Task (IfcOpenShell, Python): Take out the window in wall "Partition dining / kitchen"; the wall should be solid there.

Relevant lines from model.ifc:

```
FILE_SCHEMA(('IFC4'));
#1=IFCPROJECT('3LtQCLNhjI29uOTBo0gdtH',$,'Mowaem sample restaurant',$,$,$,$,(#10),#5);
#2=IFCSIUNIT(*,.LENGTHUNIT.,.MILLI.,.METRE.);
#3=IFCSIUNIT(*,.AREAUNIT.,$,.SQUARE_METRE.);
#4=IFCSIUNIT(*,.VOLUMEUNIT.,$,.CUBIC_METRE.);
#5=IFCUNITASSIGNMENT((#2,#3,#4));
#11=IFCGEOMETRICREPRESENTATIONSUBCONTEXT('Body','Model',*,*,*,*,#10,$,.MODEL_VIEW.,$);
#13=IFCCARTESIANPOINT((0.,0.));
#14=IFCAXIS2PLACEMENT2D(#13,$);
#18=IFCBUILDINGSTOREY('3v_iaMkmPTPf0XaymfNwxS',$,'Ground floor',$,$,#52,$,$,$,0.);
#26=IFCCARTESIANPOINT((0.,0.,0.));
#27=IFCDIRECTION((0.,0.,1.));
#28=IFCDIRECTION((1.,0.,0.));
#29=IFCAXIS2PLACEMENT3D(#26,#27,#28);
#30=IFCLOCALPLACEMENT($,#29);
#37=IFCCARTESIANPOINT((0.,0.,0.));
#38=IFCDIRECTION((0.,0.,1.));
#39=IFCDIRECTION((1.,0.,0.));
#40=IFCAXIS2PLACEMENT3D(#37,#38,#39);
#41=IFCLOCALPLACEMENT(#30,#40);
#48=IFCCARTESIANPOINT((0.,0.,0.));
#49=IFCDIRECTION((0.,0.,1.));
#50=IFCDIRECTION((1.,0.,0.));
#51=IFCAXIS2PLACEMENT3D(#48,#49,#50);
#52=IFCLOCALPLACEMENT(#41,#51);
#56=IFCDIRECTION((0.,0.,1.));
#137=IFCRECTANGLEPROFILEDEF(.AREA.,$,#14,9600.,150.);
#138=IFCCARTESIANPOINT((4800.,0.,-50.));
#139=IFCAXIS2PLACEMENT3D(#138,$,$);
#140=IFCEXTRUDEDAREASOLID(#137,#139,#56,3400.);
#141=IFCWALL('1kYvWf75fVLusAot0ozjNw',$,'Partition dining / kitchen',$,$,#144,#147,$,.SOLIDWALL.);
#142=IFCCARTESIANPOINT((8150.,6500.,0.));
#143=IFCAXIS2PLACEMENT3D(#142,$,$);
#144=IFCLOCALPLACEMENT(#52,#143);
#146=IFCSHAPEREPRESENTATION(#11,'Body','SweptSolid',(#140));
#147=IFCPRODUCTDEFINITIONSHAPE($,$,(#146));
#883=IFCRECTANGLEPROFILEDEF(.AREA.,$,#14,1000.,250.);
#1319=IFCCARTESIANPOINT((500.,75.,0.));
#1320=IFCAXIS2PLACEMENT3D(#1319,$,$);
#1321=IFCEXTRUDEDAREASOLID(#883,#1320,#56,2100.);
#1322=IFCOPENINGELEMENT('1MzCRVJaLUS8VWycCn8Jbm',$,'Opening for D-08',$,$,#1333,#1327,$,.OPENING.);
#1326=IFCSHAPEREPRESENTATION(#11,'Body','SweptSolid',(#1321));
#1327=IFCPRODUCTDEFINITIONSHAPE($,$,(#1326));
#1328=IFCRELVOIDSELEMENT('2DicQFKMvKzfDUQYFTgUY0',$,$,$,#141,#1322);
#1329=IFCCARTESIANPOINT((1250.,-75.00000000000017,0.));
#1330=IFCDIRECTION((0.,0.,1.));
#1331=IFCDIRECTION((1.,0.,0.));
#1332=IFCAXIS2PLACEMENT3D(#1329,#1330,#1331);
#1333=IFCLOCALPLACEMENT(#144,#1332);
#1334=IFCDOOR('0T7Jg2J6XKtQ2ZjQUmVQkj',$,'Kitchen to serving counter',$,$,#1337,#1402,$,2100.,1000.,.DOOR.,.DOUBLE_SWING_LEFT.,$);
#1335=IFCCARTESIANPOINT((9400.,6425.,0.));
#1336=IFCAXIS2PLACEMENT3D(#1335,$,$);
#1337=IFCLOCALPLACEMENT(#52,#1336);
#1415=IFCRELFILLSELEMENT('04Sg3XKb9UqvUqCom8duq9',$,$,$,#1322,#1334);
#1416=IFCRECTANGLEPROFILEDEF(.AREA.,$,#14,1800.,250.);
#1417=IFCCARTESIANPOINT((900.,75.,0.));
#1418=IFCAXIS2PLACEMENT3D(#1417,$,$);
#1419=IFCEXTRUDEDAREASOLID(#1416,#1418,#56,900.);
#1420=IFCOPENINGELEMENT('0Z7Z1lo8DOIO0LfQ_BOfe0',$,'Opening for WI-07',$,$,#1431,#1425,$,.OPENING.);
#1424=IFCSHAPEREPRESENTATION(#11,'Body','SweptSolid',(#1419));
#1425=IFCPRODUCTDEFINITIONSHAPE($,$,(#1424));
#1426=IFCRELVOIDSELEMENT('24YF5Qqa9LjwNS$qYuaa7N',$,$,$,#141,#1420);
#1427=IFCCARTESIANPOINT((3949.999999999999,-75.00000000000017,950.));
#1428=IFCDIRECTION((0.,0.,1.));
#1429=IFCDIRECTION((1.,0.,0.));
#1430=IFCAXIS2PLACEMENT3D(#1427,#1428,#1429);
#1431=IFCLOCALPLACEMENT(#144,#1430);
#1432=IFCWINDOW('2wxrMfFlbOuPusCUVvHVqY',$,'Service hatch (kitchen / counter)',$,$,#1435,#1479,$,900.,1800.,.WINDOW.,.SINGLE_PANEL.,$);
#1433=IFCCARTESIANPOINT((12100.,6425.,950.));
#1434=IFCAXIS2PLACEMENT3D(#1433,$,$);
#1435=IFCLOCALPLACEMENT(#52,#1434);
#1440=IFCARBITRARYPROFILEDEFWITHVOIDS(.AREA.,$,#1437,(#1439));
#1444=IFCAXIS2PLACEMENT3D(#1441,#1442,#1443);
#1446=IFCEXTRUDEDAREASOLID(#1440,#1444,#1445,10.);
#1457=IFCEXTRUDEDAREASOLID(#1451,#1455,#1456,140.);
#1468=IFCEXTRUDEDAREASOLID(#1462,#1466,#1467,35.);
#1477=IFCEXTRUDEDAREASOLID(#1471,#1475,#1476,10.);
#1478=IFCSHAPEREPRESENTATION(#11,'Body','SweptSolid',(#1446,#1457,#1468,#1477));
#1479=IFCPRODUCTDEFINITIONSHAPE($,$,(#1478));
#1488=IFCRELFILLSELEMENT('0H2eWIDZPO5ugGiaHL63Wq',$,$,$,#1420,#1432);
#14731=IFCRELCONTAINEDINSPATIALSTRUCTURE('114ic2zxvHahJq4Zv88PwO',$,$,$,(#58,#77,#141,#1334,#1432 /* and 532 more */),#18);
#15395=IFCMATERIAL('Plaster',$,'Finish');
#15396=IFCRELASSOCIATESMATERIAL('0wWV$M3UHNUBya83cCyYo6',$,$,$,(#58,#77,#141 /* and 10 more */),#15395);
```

```python
import ifcopenshell
import ifcopenshell.api.feature
import ifcopenshell.api.root
import ifcopenshell.geom
import ifcopenshell.util.shape

model = ifcopenshell.open("model.ifc")
settings = ifcopenshell.geom.settings()


def volume(element):
    """Net volume in cubic metres, openings subtracted."""
    shape = ifcopenshell.geom.create_shape(settings, element)
    return ifcopenshell.util.shape.get_volume(shape.geometry)


window = model.by_guid("2wxrMfFlbOuPusCUVvHVqY")
opening = window.FillsVoids[0].RelatingOpeningElement
wall = opening.VoidsElements[0].RelatingBuildingElement
before = volume(wall)

ifcopenshell.api.root.remove_product(model, product=window)
ifcopenshell.api.feature.remove_feature(model, feature=opening)

after = volume(wall)

print(f"wall volume {before:.3f} -> {after:.3f} m3")

model.write("model_rev.ifc")
```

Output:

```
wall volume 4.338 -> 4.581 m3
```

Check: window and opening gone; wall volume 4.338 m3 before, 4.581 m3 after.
